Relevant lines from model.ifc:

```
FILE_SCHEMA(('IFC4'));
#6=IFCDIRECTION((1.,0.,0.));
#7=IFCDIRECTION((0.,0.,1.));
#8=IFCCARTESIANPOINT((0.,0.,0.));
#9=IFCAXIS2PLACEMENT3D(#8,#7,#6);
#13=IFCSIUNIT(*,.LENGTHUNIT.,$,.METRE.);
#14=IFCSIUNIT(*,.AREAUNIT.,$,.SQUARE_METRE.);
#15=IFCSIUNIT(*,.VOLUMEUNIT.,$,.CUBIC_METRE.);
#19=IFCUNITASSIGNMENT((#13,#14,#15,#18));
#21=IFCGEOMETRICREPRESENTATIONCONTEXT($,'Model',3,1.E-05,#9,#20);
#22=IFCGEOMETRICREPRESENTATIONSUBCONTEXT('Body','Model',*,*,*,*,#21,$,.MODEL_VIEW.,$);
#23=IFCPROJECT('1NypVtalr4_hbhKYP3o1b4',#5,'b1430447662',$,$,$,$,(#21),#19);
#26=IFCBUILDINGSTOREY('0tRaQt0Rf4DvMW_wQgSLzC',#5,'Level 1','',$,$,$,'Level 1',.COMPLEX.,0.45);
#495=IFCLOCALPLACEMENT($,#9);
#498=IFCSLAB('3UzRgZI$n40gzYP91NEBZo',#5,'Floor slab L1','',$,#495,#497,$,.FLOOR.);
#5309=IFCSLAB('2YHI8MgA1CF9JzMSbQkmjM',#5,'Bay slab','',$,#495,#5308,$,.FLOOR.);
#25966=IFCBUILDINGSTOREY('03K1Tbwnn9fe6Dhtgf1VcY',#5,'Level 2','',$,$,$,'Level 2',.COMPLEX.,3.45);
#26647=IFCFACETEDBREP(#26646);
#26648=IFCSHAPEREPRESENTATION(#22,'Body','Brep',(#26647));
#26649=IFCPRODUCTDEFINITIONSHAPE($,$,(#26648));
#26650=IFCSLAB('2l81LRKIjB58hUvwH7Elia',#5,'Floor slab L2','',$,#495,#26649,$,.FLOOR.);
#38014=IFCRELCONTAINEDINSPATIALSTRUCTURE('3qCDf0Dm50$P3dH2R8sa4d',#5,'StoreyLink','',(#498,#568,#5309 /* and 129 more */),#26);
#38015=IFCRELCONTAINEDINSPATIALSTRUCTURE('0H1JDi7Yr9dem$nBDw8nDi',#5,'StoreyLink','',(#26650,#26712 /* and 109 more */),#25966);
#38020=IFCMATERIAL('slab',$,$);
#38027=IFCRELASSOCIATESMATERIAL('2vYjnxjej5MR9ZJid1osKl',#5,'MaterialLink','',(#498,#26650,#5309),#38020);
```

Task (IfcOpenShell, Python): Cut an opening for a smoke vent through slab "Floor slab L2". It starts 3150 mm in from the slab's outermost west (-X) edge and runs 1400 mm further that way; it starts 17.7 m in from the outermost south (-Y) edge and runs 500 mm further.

```python
import numpy as np
import ifcopenshell
import ifcopenshell.api.feature
import ifcopenshell.api.geometry
import ifcopenshell.api.root
import ifcopenshell.geom
import ifcopenshell.util.placement
import ifcopenshell.util.representation
import ifcopenshell.util.shape
import ifcopenshell.util.unit

model = ifcopenshell.open("model.ifc")
unit_scale = ifcopenshell.util.unit.calculate_unit_scale(model)
settings = ifcopenshell.geom.settings()


def volume(element):
    """Net volume in cubic metres, openings subtracted."""
    shape = ifcopenshell.geom.create_shape(settings, element)
    return ifcopenshell.util.shape.get_volume(shape.geometry)


slab = model.by_guid("2l81LRKIjB58hUvwH7Elia")
before = volume(slab)

# Extent in the slab's own axes, in metres. The edges named are its -X and -Y sides.
slab_shape = ifcopenshell.geom.create_shape(settings, slab)
vertices = ifcopenshell.util.shape.get_vertices(slab_shape.geometry)
x_min, y_min, bottom = vertices.min(axis=0)
top = vertices[:, 2].max()

opening = ifcopenshell.api.root.create_entity(model, ifc_class="IfcOpeningElement", name="Smoke vent opening", predefined_type="OPENING")
context = ifcopenshell.util.representation.get_context(model, "Model", "Body", "MODEL_VIEW")
width, depth = 1.4, 0.5
outline = [(0.0, 0.0), (width, 0.0), (width, depth), (0.0, depth), (0.0, 0.0)]
# Overshoot both faces by 50 mm so the cut is clean.
shape = ifcopenshell.api.geometry.add_slab_representation(
    model, context=context, depth=top - bottom + 0.1, polyline=outline
)
ifcopenshell.api.geometry.assign_representation(model, product=opening, representation=shape)

matrix = ifcopenshell.util.placement.get_local_placement(slab.ObjectPlacement)
matrix[:, 3] = matrix @ np.append(np.array([x_min + 3.15, y_min + 17.7, bottom - 0.05]) / unit_scale, 1.0)
ifcopenshell.api.geometry.edit_object_placement(model, product=opening, matrix=matrix, is_si=False)
ifcopenshell.api.feature.add_feature(model, feature=opening, element=slab)

after = volume(slab)

print(f"slab volume {before:.3f} -> {after:.3f} m3")

model.write("model_rev.ifc")
```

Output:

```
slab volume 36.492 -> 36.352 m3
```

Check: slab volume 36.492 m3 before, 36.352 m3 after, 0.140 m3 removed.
